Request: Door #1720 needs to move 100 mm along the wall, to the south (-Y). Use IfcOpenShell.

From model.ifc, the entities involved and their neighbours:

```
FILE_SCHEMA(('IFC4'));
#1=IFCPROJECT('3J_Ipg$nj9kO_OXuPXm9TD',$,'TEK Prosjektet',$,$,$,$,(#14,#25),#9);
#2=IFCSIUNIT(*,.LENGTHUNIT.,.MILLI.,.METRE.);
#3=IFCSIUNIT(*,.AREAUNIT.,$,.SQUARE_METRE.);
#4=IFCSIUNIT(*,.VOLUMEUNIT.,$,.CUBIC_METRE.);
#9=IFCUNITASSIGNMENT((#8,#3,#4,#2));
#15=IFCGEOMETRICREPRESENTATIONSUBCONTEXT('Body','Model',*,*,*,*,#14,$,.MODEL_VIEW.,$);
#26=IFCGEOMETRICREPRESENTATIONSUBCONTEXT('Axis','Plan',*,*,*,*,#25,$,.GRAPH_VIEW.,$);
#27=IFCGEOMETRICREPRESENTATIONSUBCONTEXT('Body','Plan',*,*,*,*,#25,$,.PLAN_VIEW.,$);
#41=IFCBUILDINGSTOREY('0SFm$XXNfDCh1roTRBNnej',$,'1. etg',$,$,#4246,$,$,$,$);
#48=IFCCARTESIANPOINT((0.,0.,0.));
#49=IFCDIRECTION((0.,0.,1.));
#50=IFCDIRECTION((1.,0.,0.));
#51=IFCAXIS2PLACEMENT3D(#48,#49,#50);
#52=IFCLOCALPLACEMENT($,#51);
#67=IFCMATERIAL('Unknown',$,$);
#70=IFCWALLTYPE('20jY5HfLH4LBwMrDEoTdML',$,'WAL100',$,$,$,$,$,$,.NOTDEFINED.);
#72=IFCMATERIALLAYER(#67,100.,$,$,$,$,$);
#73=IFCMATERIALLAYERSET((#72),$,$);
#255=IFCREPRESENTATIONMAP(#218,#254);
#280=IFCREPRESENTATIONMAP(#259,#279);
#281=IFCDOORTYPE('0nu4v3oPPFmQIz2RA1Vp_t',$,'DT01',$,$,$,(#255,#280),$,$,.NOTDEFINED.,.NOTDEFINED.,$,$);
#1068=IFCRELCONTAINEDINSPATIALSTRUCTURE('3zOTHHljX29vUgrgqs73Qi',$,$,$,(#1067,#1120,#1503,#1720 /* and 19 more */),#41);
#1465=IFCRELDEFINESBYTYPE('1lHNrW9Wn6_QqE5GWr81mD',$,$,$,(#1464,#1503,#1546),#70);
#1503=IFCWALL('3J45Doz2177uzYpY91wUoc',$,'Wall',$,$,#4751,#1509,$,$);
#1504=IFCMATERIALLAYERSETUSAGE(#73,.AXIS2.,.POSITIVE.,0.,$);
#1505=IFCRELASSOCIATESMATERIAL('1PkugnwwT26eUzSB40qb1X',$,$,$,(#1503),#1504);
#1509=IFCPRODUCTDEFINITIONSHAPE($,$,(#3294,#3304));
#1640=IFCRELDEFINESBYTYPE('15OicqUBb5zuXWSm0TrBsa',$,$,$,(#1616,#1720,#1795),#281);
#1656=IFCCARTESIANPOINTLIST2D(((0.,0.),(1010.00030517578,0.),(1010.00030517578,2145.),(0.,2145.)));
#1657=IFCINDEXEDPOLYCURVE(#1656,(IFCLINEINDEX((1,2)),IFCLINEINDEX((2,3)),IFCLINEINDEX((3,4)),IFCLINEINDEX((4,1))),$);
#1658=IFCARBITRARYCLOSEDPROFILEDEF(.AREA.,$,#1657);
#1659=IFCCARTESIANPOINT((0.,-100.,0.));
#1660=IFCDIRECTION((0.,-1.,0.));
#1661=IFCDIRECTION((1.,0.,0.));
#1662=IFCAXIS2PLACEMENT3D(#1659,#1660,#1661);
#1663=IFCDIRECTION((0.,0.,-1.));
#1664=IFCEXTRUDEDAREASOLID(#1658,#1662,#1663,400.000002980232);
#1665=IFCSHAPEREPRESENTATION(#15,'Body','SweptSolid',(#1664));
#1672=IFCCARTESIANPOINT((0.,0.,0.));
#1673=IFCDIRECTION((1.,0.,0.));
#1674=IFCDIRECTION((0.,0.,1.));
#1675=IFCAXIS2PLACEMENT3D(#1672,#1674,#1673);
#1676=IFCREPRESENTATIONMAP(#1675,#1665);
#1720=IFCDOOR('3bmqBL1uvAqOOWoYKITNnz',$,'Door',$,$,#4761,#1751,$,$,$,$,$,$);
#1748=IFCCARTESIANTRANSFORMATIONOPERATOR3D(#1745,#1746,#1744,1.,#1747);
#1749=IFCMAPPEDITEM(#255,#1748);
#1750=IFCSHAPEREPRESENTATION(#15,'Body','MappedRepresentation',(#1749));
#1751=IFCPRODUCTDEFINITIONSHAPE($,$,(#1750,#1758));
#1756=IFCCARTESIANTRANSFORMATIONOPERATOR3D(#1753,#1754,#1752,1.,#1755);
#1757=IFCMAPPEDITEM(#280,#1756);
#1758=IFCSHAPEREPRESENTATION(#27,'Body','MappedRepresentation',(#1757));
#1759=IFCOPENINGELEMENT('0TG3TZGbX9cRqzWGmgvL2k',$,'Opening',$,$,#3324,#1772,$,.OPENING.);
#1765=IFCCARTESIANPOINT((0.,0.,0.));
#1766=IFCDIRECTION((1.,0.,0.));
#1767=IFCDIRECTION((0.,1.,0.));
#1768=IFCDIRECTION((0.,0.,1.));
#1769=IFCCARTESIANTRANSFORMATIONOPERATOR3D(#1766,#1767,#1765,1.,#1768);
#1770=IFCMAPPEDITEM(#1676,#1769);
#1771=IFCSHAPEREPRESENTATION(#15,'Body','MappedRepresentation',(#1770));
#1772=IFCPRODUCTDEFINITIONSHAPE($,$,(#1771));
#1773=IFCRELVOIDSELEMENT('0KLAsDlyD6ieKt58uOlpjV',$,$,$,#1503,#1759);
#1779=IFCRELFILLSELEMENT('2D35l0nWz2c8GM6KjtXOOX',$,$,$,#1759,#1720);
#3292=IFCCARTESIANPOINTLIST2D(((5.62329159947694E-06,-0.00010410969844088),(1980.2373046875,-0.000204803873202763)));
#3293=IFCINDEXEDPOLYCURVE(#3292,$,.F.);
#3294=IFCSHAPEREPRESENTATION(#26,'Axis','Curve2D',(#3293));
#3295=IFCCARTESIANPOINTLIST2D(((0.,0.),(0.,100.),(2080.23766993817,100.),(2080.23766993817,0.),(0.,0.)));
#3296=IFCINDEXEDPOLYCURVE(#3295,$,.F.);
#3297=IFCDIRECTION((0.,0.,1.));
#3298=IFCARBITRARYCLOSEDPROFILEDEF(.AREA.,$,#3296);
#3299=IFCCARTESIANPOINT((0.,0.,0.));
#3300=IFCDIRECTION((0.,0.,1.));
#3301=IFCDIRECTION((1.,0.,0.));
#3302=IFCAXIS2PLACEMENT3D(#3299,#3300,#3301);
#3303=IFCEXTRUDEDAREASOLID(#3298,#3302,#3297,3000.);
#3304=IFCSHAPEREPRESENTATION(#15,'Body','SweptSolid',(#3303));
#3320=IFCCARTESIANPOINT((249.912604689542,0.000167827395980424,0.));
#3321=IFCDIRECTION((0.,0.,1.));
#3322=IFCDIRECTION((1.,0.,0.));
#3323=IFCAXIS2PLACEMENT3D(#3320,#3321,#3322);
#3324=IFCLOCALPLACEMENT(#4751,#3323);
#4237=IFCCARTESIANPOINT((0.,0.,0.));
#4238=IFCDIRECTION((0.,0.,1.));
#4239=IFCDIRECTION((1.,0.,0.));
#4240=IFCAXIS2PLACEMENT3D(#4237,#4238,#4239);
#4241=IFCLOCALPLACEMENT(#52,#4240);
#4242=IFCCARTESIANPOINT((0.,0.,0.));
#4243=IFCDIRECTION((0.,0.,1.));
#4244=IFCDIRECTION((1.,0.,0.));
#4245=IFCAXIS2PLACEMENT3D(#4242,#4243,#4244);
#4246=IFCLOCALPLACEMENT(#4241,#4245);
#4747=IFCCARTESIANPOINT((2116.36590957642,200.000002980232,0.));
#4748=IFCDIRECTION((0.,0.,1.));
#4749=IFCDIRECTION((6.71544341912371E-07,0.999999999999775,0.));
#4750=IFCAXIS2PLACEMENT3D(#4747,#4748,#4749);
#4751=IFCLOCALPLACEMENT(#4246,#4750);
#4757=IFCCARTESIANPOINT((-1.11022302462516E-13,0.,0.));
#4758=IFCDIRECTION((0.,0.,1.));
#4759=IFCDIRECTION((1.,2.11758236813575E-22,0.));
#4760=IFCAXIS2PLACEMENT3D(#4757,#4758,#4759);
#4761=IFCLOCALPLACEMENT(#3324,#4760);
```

```python
import ifcopenshell
import ifcopenshell.api.geometry
import ifcopenshell.util.placement
import ifcopenshell.util.unit

model = ifcopenshell.open("model.ifc")
unit_scale = ifcopenshell.util.unit.calculate_unit_scale(model)

door = model.by_guid("3bmqBL1uvAqOOWoYKITNnz")
opening = door.FillsVoids[0].RelatingOpeningElement
wall = opening.VoidsElements[0].RelatingBuildingElement

wall_matrix = ifcopenshell.util.placement.get_local_placement(wall.ObjectPlacement)
shift = wall_matrix[:3, 0] * -0.1 / unit_scale
before = ifcopenshell.util.placement.get_local_placement(door.ObjectPlacement)[:3, 3].copy()

# The door is placed relative to its opening, so it follows when the opening moves.
matrix = ifcopenshell.util.placement.get_local_placement(opening.ObjectPlacement)
matrix[:3, 3] += shift
ifcopenshell.api.geometry.edit_object_placement(
    model, product=opening, matrix=matrix, is_si=False, should_transform_children=True
)

after = ifcopenshell.util.placement.get_local_placement(door.ObjectPlacement)[:3, 3]
print("door moved by", (after - before).round(3) + 0.0)

model.write("model_updated.ifc")
```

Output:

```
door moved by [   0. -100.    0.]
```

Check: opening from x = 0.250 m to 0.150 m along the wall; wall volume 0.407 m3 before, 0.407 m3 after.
